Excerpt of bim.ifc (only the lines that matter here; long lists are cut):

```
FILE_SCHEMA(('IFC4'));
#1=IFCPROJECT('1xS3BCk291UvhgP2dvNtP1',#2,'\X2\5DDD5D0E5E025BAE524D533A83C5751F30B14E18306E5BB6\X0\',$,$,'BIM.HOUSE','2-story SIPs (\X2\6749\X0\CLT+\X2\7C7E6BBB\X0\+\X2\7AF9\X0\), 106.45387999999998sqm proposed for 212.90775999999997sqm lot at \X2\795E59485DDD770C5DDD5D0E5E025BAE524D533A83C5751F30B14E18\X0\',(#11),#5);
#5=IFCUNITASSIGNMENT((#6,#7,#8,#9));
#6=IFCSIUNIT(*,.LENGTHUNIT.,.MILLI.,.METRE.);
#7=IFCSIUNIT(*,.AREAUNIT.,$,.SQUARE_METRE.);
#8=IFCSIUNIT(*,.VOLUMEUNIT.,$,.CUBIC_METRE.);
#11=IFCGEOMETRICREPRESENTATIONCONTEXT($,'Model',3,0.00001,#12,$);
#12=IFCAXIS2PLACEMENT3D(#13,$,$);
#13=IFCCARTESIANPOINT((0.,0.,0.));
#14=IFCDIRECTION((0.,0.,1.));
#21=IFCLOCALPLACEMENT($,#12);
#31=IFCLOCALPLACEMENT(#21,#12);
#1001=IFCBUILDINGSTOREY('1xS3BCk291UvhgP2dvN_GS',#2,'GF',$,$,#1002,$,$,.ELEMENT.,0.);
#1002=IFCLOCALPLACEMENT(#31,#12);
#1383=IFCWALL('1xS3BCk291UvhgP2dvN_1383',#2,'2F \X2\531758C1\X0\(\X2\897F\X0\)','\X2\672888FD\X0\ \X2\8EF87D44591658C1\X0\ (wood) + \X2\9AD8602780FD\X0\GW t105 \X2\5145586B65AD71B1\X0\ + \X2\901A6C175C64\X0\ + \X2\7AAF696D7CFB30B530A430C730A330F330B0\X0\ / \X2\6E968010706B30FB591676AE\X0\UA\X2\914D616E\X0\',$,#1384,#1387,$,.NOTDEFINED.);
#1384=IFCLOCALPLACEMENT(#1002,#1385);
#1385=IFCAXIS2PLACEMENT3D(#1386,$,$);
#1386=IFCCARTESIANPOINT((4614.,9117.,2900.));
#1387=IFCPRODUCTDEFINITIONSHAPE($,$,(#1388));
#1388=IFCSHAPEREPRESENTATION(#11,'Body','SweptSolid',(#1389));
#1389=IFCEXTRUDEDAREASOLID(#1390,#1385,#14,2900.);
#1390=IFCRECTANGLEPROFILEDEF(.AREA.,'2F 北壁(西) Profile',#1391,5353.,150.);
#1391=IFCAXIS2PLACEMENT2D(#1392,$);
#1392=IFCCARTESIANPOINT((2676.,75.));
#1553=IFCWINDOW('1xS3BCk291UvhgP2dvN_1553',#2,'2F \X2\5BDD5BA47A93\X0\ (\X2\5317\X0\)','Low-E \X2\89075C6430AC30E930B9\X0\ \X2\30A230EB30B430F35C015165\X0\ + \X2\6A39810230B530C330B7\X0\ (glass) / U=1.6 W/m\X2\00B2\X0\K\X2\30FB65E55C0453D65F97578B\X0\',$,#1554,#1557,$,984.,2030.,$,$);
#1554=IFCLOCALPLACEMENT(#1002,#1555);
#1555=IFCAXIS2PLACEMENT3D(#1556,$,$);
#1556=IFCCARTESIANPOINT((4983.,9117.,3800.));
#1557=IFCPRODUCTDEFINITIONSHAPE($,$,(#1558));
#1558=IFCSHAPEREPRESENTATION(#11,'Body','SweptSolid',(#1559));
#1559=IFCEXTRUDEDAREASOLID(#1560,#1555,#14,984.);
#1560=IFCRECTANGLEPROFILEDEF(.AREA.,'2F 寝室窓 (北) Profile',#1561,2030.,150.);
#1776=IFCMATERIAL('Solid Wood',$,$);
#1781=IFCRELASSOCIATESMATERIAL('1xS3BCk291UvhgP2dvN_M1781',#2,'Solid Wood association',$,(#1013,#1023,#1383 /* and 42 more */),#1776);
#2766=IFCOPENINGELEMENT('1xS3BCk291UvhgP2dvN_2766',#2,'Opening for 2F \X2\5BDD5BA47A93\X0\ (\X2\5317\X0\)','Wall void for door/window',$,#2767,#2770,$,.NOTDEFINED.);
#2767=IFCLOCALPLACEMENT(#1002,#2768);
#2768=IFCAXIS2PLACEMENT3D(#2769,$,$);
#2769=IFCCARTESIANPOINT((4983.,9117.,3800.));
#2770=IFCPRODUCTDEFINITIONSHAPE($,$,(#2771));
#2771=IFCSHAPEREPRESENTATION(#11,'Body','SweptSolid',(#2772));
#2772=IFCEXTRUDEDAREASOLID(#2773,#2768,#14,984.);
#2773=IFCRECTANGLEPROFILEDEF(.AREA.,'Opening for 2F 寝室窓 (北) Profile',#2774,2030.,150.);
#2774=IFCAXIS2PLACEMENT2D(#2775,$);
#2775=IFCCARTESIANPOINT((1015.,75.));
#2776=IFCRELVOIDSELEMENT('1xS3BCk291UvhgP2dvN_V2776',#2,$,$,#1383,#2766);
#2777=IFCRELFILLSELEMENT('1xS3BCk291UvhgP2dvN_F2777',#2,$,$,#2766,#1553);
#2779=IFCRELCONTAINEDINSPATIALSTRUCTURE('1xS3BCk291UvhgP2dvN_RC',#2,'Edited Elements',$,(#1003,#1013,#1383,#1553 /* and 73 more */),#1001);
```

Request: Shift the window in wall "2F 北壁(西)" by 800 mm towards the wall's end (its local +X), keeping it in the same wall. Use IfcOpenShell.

```python
import ifcopenshell
import ifcopenshell.api.geometry
import ifcopenshell.util.placement
import ifcopenshell.util.unit

model = ifcopenshell.open("bim.ifc")
unit_scale = ifcopenshell.util.unit.calculate_unit_scale(model)

window = model.by_guid("1xS3BCk291UvhgP2dvN_1553")
opening = window.FillsVoids[0].RelatingOpeningElement
wall = opening.VoidsElements[0].RelatingBuildingElement

wall_matrix = ifcopenshell.util.placement.get_local_placement(wall.ObjectPlacement)
shift = wall_matrix[:3, 0] * 0.8 / unit_scale
before = ifcopenshell.util.placement.get_local_placement(window.ObjectPlacement)[:3, 3].copy()

# The window is not placed relative to its opening, so move both.
for product in (opening, window):
    matrix = ifcopenshell.util.placement.get_local_placement(product.ObjectPlacement)
    matrix[:3, 3] += shift
    ifcopenshell.api.geometry.edit_object_placement(model, product=product, matrix=matrix, is_si=False)

after = ifcopenshell.util.placement.get_local_placement(window.ObjectPlacement)[:3, 3]
print("window moved by", (after - before).round(3) + 0.0)

model.write("bim_rev.ifc")
```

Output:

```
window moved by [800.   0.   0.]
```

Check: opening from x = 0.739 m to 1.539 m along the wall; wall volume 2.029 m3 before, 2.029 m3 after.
